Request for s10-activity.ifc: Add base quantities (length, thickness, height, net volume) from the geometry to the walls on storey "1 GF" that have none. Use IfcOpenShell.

First a look at what the model holds.

```python
import ifcopenshell
import ifcopenshell.util.element
import ifcopenshell.util.unit

model = ifcopenshell.open("s10-activity.ifc")
print(model.schema)
for unit_type in ("LENGTHUNIT", "AREAUNIT", "VOLUMEUNIT"):
    print(unit_type, ifcopenshell.util.unit.calculate_unit_scale(model, unit_type))
storey = next(s for s in model.by_type("IfcBuildingStorey") if s.Name == "1 GF")
walls = [e for e in ifcopenshell.util.element.get_decomposition(storey) if e.is_a("IfcWall")]
for e in sorted(walls, key=lambda e: e.id()):
    print(e.id(), e.is_a(), e.Name, list(ifcopenshell.util.element.get_psets(e, qtos_only=True)), sep=" | ")
```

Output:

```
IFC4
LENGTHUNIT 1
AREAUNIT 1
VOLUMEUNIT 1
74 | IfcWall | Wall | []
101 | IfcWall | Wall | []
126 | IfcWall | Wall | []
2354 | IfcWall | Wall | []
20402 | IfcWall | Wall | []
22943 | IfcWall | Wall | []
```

```python
import ifcopenshell
import ifcopenshell.api.pset
import ifcopenshell.geom
import ifcopenshell.util.element
import ifcopenshell.util.shape
import ifcopenshell.util.unit

model = ifcopenshell.open("s10-activity.ifc")
unit_scale = ifcopenshell.util.unit.calculate_unit_scale(model)
volume_scale = ifcopenshell.util.unit.calculate_unit_scale(model, "VOLUMEUNIT")
settings = ifcopenshell.geom.settings()

storey = next(s for s in model.by_type("IfcBuildingStorey") if s.Name == "1 GF")
walls = [e for e in ifcopenshell.util.element.get_decomposition(storey) if e.is_a("IfcWall")]

for e in sorted(walls, key=lambda e: e.id()):
    if ifcopenshell.util.element.get_psets(e, qtos_only=True, should_inherit=False):
        continue
    # Geometry comes back in metres, in the element's own axes.
    shape = ifcopenshell.geom.create_shape(settings, e)
    values = {
        "Length": ifcopenshell.util.shape.get_x(shape.geometry) / unit_scale,
        "Width": ifcopenshell.util.shape.get_y(shape.geometry) / unit_scale,
        "Height": ifcopenshell.util.shape.get_z(shape.geometry) / unit_scale,
        "NetVolume": ifcopenshell.util.shape.get_volume(shape.geometry) / volume_scale,
    }
    qto = ifcopenshell.api.pset.add_qto(model, product=e, name="Qto_WallBaseQuantities")
    ifcopenshell.api.pset.edit_qto(model, qto=qto, properties=values)
    print(e.id(), {k: round(v, 3) for k, v in values.items()})

model.write("s10-activity_v2.ifc")
```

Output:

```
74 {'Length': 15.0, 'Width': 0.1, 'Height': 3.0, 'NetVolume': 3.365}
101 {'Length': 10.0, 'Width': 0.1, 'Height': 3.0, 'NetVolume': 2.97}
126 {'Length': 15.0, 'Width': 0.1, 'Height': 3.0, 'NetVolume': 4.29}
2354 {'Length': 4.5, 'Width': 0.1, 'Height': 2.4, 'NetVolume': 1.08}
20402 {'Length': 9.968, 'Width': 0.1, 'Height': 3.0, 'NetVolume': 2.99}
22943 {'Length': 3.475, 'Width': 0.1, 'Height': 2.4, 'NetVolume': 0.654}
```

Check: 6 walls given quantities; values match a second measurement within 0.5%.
